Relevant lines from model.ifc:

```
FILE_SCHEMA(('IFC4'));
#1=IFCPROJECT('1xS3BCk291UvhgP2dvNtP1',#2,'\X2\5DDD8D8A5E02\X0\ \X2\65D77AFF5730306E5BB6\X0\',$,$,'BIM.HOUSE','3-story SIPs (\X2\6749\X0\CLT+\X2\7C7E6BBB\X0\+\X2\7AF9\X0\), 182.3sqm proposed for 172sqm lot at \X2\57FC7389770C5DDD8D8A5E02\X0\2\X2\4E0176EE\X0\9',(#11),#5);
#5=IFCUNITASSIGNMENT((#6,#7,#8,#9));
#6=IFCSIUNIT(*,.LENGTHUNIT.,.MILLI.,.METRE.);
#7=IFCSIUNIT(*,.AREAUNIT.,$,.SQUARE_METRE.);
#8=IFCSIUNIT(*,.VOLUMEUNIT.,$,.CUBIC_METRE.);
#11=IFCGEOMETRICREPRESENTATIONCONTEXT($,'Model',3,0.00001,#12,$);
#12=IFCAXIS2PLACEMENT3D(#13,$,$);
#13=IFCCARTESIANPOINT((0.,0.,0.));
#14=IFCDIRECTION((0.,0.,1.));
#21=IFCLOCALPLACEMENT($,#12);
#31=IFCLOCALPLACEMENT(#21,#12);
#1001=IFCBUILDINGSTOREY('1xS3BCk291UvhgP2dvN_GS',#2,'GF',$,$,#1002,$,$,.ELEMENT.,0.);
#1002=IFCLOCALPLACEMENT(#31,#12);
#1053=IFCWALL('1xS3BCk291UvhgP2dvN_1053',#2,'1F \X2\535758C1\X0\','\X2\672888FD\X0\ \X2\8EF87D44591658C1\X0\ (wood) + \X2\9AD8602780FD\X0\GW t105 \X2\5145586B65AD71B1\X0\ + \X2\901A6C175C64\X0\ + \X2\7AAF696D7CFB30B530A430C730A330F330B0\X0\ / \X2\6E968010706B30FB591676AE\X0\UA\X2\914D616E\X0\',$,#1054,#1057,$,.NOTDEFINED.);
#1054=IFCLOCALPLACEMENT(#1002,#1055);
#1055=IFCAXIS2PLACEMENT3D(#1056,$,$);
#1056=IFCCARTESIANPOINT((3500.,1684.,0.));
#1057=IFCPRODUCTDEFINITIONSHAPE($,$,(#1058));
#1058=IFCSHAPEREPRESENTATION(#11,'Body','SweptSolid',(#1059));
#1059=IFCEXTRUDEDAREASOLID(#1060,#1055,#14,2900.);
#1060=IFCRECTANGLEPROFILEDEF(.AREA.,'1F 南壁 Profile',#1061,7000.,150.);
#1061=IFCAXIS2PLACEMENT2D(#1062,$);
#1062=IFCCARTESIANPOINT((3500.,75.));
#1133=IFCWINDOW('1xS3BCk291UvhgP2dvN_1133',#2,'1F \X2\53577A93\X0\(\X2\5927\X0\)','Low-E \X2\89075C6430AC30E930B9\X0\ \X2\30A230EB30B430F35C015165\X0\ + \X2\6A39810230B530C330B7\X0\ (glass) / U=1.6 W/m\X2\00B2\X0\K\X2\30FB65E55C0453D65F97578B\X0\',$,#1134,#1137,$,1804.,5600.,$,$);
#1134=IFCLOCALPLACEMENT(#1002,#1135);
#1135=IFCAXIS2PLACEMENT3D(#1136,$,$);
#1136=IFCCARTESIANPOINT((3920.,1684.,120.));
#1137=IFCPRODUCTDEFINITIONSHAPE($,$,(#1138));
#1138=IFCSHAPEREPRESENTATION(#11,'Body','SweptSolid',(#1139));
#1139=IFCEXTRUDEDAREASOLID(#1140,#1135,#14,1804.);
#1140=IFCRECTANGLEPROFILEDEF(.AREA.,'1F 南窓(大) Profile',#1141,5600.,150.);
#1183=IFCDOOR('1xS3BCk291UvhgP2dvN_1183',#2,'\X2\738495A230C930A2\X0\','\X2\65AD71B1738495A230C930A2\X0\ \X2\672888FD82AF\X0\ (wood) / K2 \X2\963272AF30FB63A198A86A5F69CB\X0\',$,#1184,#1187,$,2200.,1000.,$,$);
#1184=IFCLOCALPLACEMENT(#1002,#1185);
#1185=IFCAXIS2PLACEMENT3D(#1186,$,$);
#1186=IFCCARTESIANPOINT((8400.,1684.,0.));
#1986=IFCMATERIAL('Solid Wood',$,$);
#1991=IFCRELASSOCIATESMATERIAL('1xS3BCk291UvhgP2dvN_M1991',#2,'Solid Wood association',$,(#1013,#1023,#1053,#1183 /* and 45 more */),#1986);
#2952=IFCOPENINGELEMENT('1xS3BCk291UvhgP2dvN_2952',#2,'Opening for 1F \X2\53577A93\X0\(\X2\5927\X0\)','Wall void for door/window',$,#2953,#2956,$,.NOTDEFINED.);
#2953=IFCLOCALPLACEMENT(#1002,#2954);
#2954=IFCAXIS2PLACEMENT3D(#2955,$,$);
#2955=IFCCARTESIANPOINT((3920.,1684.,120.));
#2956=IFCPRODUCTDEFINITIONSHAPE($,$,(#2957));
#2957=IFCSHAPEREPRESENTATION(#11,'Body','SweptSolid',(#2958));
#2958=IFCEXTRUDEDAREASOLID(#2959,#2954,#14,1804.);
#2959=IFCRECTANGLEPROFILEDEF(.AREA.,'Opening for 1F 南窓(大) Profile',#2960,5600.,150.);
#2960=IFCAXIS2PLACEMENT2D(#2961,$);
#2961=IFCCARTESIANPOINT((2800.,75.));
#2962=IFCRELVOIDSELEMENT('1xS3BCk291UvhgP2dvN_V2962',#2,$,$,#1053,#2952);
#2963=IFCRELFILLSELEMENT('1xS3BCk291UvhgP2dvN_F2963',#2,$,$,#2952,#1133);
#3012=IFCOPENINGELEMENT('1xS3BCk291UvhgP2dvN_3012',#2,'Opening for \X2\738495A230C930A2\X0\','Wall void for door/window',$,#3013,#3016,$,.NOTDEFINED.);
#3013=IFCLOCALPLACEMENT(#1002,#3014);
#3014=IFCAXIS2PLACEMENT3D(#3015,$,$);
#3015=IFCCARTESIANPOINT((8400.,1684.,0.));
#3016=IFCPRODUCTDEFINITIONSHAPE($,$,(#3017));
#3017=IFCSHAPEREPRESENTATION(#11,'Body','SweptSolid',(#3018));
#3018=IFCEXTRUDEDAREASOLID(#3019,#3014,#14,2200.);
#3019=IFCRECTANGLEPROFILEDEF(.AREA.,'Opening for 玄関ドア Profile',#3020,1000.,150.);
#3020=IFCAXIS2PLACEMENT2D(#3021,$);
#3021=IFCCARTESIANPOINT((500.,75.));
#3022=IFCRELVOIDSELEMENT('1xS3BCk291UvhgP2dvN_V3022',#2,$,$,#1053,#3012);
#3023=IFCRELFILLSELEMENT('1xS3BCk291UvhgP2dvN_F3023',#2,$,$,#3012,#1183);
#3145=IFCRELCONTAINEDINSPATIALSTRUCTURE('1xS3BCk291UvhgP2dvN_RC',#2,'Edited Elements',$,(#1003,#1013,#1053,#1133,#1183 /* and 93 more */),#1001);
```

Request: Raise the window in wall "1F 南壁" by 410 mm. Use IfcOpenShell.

```python
import numpy as np
import ifcopenshell
import ifcopenshell.api.geometry
import ifcopenshell.util.placement
import ifcopenshell.util.unit

model = ifcopenshell.open("model.ifc")
unit_scale = ifcopenshell.util.unit.calculate_unit_scale(model)

window = model.by_guid("1xS3BCk291UvhgP2dvN_1133")
opening = window.FillsVoids[0].RelatingOpeningElement
dz = 410.0

shift = np.array([0.0, 0.0, dz])
# The window is not placed relative to its opening, so move both.
for product in (opening, window):
    matrix = ifcopenshell.util.placement.get_local_placement(product.ObjectPlacement)
    matrix[:3, 3] += shift
    ifcopenshell.api.geometry.edit_object_placement(model, product=product, matrix=matrix, is_si=False)

print(f"moved by {dz * unit_scale:+.3f} m")

model.write("model_rev.ifc")
```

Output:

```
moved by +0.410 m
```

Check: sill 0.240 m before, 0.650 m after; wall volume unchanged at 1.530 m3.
